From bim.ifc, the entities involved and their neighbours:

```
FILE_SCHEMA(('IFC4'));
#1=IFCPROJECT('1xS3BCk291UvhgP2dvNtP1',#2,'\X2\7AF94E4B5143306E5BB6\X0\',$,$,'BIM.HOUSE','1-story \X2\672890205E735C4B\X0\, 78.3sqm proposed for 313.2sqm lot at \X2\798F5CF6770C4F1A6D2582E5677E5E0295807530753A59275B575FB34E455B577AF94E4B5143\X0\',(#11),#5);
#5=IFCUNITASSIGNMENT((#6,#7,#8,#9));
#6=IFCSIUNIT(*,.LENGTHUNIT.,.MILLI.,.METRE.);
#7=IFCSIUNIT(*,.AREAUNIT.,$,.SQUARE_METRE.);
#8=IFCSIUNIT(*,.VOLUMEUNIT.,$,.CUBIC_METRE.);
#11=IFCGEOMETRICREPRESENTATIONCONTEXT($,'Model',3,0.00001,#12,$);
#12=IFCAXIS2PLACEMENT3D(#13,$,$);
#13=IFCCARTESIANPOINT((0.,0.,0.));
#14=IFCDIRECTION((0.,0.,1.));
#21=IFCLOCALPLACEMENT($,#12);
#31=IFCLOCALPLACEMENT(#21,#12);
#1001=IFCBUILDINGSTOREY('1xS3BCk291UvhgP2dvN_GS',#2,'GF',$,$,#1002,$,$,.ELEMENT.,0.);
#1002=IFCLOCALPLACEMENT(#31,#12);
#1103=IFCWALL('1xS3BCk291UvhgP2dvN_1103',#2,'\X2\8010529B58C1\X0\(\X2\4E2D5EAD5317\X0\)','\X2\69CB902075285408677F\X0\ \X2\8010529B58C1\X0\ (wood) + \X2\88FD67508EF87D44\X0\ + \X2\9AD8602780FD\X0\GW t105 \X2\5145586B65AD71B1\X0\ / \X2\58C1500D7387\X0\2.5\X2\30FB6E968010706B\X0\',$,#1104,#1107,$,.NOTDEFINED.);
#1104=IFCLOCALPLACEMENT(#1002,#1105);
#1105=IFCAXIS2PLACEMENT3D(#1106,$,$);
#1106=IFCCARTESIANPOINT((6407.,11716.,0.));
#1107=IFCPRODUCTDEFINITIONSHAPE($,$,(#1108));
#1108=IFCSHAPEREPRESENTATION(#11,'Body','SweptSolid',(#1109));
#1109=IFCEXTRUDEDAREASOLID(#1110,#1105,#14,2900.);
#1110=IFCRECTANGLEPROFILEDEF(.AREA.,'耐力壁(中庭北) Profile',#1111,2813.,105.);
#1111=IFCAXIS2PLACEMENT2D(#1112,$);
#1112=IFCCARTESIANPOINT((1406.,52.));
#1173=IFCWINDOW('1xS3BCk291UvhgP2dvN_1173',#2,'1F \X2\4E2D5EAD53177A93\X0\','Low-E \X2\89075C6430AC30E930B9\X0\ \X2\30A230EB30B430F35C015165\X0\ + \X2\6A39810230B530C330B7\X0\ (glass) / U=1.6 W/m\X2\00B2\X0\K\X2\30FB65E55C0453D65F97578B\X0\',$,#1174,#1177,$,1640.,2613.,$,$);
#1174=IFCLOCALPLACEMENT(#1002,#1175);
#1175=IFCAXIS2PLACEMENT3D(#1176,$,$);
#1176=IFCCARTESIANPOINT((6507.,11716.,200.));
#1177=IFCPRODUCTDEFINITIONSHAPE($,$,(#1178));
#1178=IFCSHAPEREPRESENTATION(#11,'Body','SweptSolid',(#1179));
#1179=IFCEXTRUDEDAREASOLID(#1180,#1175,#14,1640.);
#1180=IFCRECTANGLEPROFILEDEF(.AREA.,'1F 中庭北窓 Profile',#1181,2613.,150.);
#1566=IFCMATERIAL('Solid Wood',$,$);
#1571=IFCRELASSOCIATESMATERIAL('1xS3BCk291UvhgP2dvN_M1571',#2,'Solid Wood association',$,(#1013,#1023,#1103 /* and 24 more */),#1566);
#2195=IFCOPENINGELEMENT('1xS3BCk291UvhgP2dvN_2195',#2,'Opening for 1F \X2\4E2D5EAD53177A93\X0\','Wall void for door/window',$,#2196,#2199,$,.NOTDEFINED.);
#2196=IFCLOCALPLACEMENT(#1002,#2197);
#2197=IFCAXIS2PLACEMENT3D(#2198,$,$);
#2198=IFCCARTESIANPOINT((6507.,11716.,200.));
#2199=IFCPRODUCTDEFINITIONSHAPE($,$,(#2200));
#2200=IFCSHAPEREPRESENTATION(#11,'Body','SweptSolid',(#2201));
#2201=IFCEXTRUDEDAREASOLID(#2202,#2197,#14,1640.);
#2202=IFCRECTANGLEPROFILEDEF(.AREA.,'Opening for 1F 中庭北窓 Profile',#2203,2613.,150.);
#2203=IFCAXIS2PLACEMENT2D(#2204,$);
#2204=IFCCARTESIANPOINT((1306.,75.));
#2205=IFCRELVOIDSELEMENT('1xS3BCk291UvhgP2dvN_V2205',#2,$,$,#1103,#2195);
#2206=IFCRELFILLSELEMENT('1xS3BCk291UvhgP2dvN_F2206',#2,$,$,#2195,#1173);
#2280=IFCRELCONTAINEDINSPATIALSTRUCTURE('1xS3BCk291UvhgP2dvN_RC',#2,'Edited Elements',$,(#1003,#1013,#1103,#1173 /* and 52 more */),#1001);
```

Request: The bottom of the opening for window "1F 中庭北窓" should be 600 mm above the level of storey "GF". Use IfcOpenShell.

```python
import numpy as np
import ifcopenshell
import ifcopenshell.api.geometry
import ifcopenshell.geom
import ifcopenshell.util.element
import ifcopenshell.util.placement
import ifcopenshell.util.shape
import ifcopenshell.util.unit

model = ifcopenshell.open("bim.ifc")
unit_scale = ifcopenshell.util.unit.calculate_unit_scale(model)

window = model.by_guid("1xS3BCk291UvhgP2dvN_1173")
opening = window.FillsVoids[0].RelatingOpeningElement
storey = ifcopenshell.util.element.get_container(window, ifc_class="IfcBuildingStorey")
level = ifcopenshell.util.placement.get_local_placement(storey.ObjectPlacement)[2, 3]

# The opening's origin need not be at the sill, so measure its lowest point.
shape = ifcopenshell.geom.create_shape(ifcopenshell.geom.settings(), opening)
bottom = ifcopenshell.util.shape.get_shape_bottom_elevation(shape, shape.geometry) / unit_scale
dz = level + 0.6 / unit_scale - bottom

shift = np.array([0.0, 0.0, dz])
# The window is not placed relative to its opening, so move both.
for product in (opening, window):
    matrix = ifcopenshell.util.placement.get_local_placement(product.ObjectPlacement)
    matrix[:3, 3] += shift
    ifcopenshell.api.geometry.edit_object_placement(model, product=product, matrix=matrix, is_si=False)

print(f"moved by {dz * unit_scale:+.3f} m")

model.write("bim_updated.ifc")
```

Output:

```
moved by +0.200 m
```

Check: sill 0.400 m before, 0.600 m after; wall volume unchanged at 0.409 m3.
